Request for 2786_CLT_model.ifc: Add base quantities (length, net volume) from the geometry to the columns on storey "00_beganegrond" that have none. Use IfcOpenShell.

First a look at what the model holds.

```python
import ifcopenshell
import ifcopenshell.util.element
import ifcopenshell.util.unit

model = ifcopenshell.open("2786_CLT_model.ifc")
print(model.schema)
for unit_type in ("LENGTHUNIT", "AREAUNIT", "VOLUMEUNIT"):
    print(unit_type, ifcopenshell.util.unit.calculate_unit_scale(model, unit_type))
storey = next(s for s in model.by_type("IfcBuildingStorey") if s.Name == "00_beganegrond")
columns = [e for e in ifcopenshell.util.element.get_decomposition(storey) if e.is_a("IfcColumn")]
for e in sorted(columns, key=lambda e: e.id()):
    print(e.id(), e.is_a(), e.Name, list(ifcopenshell.util.element.get_psets(e, qtos_only=True)), sep=" | ")
```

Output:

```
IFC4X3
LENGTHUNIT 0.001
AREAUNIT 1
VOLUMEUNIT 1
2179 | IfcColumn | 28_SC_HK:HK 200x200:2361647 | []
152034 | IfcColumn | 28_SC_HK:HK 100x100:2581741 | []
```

```python
import ifcopenshell
import ifcopenshell.api.pset
import ifcopenshell.geom
import ifcopenshell.util.element
import ifcopenshell.util.shape
import ifcopenshell.util.unit

model = ifcopenshell.open("2786_CLT_model.ifc")
unit_scale = ifcopenshell.util.unit.calculate_unit_scale(model)
volume_scale = ifcopenshell.util.unit.calculate_unit_scale(model, "VOLUMEUNIT")
settings = ifcopenshell.geom.settings()

storey = next(s for s in model.by_type("IfcBuildingStorey") if s.Name == "00_beganegrond")
columns = [e for e in ifcopenshell.util.element.get_decomposition(storey) if e.is_a("IfcColumn")]

for e in sorted(columns, key=lambda e: e.id()):
    if ifcopenshell.util.element.get_psets(e, qtos_only=True, should_inherit=False):
        continue
    # Geometry comes back in metres, in the element's own axes.
    shape = ifcopenshell.geom.create_shape(settings, e)
    values = {
        "Length": ifcopenshell.util.shape.get_z(shape.geometry) / unit_scale,
        "NetVolume": ifcopenshell.util.shape.get_volume(shape.geometry) / volume_scale,
    }
    qto = ifcopenshell.api.pset.add_qto(model, product=e, name="Qto_ColumnBaseQuantities")
    ifcopenshell.api.pset.edit_qto(model, qto=qto, properties=values)
    print(e.id(), {k: round(v, 3) for k, v in values.items()})

model.write("2786_CLT_model_rev.ifc")
```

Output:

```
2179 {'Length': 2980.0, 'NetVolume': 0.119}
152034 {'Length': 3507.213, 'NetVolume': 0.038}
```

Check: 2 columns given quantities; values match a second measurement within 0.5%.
